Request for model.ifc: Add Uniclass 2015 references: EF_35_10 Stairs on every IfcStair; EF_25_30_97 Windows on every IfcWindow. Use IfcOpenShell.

First a look at what the model holds.

```python
import ifcopenshell

model = ifcopenshell.open("model.ifc")
print(model.schema)
print("classifications:", [c.Name for c in model.by_type("IfcClassification")])
for ifc_class in ("IfcDoor", "IfcRoof", "IfcStair", "IfcWall", "IfcWindow"):
    print(ifc_class, len(model.by_type(ifc_class)))
```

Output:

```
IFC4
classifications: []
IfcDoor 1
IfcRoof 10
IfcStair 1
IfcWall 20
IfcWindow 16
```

```python
import ifcopenshell
import ifcopenshell.api.classification

model = ifcopenshell.open("model.ifc")

system = ifcopenshell.api.classification.add_classification(model, classification="Uniclass 2015")

codes = {
    "IfcStair": ("EF_35_10", "Stairs"),
    "IfcWindow": ("EF_25_30_97", "Windows"),
}
for ifc_class, (code, name) in codes.items():
    products = model.by_type(ifc_class)
    ifcopenshell.api.classification.add_reference(
        model, products=products, classification=system, identification=code, name=name
    )
    print(code, len(products))

model.write("model-out.ifc")
```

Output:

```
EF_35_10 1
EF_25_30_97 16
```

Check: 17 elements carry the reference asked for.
